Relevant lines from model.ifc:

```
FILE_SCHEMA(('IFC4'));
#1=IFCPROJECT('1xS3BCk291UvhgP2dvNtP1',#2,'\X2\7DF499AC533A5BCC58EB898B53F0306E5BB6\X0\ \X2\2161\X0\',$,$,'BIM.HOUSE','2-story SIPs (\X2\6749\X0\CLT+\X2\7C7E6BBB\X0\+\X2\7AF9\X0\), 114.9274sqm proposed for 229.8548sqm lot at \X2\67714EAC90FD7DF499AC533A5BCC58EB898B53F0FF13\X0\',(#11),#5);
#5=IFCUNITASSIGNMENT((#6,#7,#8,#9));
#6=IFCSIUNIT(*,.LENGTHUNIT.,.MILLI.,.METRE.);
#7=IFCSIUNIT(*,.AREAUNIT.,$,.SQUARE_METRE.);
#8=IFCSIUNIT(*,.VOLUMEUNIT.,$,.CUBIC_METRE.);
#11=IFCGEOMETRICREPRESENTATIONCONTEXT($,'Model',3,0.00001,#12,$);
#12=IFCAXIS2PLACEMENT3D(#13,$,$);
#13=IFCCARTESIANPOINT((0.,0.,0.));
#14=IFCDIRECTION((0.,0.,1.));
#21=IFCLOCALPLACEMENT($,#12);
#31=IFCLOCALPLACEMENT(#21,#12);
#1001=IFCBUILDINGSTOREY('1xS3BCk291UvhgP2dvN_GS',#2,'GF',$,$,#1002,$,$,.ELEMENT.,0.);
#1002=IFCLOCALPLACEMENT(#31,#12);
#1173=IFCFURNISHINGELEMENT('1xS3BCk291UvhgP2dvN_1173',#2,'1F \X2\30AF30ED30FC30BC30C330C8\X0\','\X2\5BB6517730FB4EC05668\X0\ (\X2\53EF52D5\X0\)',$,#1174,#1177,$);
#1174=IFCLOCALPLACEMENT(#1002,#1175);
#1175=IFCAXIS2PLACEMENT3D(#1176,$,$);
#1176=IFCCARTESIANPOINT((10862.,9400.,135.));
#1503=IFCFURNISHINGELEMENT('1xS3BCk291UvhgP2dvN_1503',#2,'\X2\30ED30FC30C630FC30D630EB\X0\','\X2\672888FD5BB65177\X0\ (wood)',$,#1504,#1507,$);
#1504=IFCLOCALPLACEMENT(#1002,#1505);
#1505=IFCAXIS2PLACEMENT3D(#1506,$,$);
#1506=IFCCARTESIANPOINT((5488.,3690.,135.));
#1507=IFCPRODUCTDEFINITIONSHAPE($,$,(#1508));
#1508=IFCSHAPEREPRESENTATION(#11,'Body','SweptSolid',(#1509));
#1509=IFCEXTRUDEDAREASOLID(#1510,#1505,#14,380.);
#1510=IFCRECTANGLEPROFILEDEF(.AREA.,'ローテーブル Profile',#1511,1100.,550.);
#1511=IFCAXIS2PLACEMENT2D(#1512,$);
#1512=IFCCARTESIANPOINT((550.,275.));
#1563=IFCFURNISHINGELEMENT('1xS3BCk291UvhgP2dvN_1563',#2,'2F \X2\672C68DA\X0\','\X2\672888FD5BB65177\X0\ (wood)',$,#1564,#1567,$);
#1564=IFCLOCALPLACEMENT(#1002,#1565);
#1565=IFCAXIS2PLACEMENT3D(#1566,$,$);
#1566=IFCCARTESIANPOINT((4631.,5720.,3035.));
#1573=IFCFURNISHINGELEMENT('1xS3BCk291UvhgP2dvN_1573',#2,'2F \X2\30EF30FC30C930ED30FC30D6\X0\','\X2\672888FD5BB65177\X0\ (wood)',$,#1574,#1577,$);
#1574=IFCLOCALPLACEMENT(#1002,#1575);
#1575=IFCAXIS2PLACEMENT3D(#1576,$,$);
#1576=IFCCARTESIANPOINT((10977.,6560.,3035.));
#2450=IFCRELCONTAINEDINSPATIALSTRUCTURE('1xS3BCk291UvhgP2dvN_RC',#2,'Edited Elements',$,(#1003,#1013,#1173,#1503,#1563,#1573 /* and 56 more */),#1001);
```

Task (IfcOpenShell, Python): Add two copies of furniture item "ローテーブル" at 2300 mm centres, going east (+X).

```python
import numpy as np
import ifcopenshell
import ifcopenshell.api.geometry
import ifcopenshell.api.root
import ifcopenshell.util.element
import ifcopenshell.util.placement
import ifcopenshell.util.unit

model = ifcopenshell.open("model.ifc")
unit_scale = ifcopenshell.util.unit.calculate_unit_scale(model)


def reuse_history(source, copy):
    """copy_class also copies each property set's owner history, people and application; keep the originals."""
    for rel in copy.IsDefinedBy:
        if rel.is_a("IfcRelDefinesByProperties") and (history := rel.RelatingPropertyDefinition.OwnerHistory):
            rel.RelatingPropertyDefinition.OwnerHistory = source.OwnerHistory
            ifcopenshell.util.element.remove_deep2(model, history)


source = model.by_id(1503)
base = ifcopenshell.util.placement.get_local_placement(source.ObjectPlacement)
step = np.array([1.0, 0.0, 0.0]) * 2.3 / unit_scale

for i in range(1, 3):
    copy = ifcopenshell.api.root.copy_class(model, product=source)
    copy.Representation = ifcopenshell.util.element.copy_deep(
        model, source.Representation, exclude=["IfcGeometricRepresentationContext", "IfcRepresentationMap"]
    )
    reuse_history(source, copy)
    matrix = base.copy()
    matrix[:3, 3] += i * step
    print("added at", matrix[:3, 3].round(3) + 0.0)
    ifcopenshell.api.geometry.edit_object_placement(model, product=copy, matrix=matrix, is_si=False)

model.write("model_rev.ifc")
```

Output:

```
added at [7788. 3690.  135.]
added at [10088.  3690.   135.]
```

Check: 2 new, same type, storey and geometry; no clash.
